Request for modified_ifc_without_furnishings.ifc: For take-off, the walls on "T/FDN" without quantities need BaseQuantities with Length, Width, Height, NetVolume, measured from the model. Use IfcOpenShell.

First a look at what the model holds.

```python
import ifcopenshell
import ifcopenshell.util.element
import ifcopenshell.util.unit

model = ifcopenshell.open("modified_ifc_without_furnishings.ifc")
print(model.schema)
for unit_type in ("LENGTHUNIT", "AREAUNIT", "VOLUMEUNIT"):
    print(unit_type, ifcopenshell.util.unit.calculate_unit_scale(model, unit_type))
storey = next(s for s in model.by_type("IfcBuildingStorey") if s.Name == "T/FDN")
walls = [e for e in ifcopenshell.util.element.get_decomposition(storey) if e.is_a("IfcWall")]
for e in sorted(walls, key=lambda e: e.id()):
    print(e.id(), e.is_a(), e.Name, list(ifcopenshell.util.element.get_psets(e, qtos_only=True)), sep=" | ")
```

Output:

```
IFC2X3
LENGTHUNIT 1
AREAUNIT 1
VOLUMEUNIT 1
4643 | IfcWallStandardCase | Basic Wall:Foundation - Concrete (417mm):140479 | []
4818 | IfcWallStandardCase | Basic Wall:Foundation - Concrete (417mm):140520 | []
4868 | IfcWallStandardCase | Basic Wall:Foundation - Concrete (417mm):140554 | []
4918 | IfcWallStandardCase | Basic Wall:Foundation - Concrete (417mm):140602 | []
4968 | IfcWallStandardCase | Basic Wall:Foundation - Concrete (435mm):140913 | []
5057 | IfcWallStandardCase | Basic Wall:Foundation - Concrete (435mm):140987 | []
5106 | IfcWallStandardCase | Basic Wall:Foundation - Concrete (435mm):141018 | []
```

```python
import ifcopenshell
import ifcopenshell.api.pset
import ifcopenshell.geom
import ifcopenshell.util.element
import ifcopenshell.util.shape
import ifcopenshell.util.unit

model = ifcopenshell.open("modified_ifc_without_furnishings.ifc")
unit_scale = ifcopenshell.util.unit.calculate_unit_scale(model)
volume_scale = ifcopenshell.util.unit.calculate_unit_scale(model, "VOLUMEUNIT")
settings = ifcopenshell.geom.settings()

storey = next(s for s in model.by_type("IfcBuildingStorey") if s.Name == "T/FDN")
walls = [e for e in ifcopenshell.util.element.get_decomposition(storey) if e.is_a("IfcWall")]

for e in sorted(walls, key=lambda e: e.id()):
    if ifcopenshell.util.element.get_psets(e, qtos_only=True, should_inherit=False):
        continue
    # Geometry comes back in metres, in the element's own axes.
    shape = ifcopenshell.geom.create_shape(settings, e)
    values = {
        "Length": ifcopenshell.util.shape.get_x(shape.geometry) / unit_scale,
        "Width": ifcopenshell.util.shape.get_y(shape.geometry) / unit_scale,
        "Height": ifcopenshell.util.shape.get_z(shape.geometry) / unit_scale,
        "NetVolume": ifcopenshell.util.shape.get_volume(shape.geometry) / volume_scale,
    }
    qto = ifcopenshell.api.pset.add_qto(model, product=e, name="BaseQuantities")
    ifcopenshell.api.pset.edit_qto(model, qto=qto, properties=values)
    print(e.id(), {k: round(v, 3) for k, v in values.items()})

model.write("modified_ifc_without_furnishings_rev.ifc")
```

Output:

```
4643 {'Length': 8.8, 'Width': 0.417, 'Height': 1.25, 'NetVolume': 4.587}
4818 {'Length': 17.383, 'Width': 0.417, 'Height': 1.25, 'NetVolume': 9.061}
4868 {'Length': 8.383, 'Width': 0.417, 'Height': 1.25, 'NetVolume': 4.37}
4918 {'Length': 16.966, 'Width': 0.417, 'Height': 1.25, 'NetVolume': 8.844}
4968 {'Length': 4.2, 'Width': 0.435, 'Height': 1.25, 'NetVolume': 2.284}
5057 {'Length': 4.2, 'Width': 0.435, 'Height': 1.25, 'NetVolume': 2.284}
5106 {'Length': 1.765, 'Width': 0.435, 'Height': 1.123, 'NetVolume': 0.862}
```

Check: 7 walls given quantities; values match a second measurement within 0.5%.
